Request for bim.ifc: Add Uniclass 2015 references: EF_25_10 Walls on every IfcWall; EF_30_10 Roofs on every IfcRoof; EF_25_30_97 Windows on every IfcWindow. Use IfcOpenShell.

First a look at what the model holds.

```python
import ifcopenshell

model = ifcopenshell.open("bim.ifc")
print(model.schema)
print("classifications:", [c.Name for c in model.by_type("IfcClassification")])
for ifc_class in ("IfcDoor", "IfcRoof", "IfcStair", "IfcWall", "IfcWindow"):
    print(ifc_class, len(model.by_type(ifc_class)))
```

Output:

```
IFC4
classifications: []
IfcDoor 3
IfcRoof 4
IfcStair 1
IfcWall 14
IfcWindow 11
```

```python
import ifcopenshell
import ifcopenshell.api.classification

model = ifcopenshell.open("bim.ifc")

system = ifcopenshell.api.classification.add_classification(model, classification="Uniclass 2015")

codes = {
    "IfcWall": ("EF_25_10", "Walls"),
    "IfcRoof": ("EF_30_10", "Roofs"),
    "IfcWindow": ("EF_25_30_97", "Windows"),
}
for ifc_class, (code, name) in codes.items():
    products = model.by_type(ifc_class)
    ifcopenshell.api.classification.add_reference(
        model, products=products, classification=system, identification=code, name=name
    )
    print(code, len(products))

model.write("bim_v2.ifc")
```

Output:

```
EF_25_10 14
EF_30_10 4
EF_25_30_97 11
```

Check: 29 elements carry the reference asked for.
